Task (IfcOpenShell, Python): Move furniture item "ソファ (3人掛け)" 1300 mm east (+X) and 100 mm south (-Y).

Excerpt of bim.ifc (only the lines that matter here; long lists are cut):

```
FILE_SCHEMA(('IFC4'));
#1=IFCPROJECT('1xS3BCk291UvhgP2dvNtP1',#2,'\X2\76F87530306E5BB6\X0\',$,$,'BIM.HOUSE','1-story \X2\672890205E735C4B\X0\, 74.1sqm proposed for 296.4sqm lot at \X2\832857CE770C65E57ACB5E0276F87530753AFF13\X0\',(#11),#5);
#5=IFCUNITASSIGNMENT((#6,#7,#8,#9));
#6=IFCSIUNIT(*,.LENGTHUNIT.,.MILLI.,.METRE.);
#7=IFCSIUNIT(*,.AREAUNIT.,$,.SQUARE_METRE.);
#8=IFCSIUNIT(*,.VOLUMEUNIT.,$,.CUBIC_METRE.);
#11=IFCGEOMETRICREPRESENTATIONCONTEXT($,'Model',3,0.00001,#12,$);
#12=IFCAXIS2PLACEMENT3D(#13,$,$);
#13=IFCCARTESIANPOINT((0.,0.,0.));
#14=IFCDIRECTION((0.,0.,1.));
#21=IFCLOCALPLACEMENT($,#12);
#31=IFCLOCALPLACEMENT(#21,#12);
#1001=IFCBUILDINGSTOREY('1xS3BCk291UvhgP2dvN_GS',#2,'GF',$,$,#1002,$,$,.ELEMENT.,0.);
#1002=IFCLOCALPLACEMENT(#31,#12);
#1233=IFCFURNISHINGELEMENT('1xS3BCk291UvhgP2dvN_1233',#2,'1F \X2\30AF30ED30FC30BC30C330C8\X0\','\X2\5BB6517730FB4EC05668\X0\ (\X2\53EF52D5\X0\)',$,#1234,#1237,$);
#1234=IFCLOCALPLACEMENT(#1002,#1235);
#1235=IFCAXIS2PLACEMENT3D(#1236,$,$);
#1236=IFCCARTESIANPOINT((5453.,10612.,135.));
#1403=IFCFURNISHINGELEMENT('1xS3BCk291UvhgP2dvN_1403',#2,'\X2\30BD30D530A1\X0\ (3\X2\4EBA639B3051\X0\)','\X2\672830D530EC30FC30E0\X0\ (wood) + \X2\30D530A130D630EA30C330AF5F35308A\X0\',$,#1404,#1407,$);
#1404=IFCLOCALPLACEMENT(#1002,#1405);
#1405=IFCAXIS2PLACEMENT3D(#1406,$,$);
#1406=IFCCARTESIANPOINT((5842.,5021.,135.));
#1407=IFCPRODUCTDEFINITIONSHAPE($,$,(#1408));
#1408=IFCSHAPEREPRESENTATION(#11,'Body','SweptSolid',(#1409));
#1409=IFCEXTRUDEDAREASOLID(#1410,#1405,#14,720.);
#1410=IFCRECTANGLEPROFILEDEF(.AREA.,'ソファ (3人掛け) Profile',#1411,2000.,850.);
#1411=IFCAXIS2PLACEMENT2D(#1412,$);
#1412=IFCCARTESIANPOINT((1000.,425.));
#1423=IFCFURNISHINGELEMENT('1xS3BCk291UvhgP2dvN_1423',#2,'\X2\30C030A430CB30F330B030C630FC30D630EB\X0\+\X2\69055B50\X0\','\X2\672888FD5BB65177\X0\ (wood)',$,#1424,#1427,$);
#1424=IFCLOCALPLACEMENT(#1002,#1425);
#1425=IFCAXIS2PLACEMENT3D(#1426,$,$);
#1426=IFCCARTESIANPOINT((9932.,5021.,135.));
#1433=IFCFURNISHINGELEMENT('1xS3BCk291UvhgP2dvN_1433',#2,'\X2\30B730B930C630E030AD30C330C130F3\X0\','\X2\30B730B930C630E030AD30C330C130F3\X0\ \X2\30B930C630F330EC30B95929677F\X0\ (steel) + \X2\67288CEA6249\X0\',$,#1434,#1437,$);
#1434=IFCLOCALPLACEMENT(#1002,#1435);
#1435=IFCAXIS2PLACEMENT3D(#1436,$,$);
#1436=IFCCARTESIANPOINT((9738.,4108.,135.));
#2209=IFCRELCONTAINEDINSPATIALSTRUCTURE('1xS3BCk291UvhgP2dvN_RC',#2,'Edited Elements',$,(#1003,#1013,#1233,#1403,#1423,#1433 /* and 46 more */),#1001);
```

```python
import ifcopenshell
import ifcopenshell.api.geometry
import ifcopenshell.util.placement

model = ifcopenshell.open("bim.ifc")

item = model.by_guid("1xS3BCk291UvhgP2dvN_1403")
matrix = ifcopenshell.util.placement.get_local_placement(item.ObjectPlacement)
matrix[0, 3] += 1300.0
matrix[1, 3] -= 100.0
ifcopenshell.api.geometry.edit_object_placement(model, product=item, matrix=matrix, is_si=False)

print(ifcopenshell.util.placement.get_local_placement(item.ObjectPlacement).round(3) + 0.0)

model.write("bim_v2.ifc")
```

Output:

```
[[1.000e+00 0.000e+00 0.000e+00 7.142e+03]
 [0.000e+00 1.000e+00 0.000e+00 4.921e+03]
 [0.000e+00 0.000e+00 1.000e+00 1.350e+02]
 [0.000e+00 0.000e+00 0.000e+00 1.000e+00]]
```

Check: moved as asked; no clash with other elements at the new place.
